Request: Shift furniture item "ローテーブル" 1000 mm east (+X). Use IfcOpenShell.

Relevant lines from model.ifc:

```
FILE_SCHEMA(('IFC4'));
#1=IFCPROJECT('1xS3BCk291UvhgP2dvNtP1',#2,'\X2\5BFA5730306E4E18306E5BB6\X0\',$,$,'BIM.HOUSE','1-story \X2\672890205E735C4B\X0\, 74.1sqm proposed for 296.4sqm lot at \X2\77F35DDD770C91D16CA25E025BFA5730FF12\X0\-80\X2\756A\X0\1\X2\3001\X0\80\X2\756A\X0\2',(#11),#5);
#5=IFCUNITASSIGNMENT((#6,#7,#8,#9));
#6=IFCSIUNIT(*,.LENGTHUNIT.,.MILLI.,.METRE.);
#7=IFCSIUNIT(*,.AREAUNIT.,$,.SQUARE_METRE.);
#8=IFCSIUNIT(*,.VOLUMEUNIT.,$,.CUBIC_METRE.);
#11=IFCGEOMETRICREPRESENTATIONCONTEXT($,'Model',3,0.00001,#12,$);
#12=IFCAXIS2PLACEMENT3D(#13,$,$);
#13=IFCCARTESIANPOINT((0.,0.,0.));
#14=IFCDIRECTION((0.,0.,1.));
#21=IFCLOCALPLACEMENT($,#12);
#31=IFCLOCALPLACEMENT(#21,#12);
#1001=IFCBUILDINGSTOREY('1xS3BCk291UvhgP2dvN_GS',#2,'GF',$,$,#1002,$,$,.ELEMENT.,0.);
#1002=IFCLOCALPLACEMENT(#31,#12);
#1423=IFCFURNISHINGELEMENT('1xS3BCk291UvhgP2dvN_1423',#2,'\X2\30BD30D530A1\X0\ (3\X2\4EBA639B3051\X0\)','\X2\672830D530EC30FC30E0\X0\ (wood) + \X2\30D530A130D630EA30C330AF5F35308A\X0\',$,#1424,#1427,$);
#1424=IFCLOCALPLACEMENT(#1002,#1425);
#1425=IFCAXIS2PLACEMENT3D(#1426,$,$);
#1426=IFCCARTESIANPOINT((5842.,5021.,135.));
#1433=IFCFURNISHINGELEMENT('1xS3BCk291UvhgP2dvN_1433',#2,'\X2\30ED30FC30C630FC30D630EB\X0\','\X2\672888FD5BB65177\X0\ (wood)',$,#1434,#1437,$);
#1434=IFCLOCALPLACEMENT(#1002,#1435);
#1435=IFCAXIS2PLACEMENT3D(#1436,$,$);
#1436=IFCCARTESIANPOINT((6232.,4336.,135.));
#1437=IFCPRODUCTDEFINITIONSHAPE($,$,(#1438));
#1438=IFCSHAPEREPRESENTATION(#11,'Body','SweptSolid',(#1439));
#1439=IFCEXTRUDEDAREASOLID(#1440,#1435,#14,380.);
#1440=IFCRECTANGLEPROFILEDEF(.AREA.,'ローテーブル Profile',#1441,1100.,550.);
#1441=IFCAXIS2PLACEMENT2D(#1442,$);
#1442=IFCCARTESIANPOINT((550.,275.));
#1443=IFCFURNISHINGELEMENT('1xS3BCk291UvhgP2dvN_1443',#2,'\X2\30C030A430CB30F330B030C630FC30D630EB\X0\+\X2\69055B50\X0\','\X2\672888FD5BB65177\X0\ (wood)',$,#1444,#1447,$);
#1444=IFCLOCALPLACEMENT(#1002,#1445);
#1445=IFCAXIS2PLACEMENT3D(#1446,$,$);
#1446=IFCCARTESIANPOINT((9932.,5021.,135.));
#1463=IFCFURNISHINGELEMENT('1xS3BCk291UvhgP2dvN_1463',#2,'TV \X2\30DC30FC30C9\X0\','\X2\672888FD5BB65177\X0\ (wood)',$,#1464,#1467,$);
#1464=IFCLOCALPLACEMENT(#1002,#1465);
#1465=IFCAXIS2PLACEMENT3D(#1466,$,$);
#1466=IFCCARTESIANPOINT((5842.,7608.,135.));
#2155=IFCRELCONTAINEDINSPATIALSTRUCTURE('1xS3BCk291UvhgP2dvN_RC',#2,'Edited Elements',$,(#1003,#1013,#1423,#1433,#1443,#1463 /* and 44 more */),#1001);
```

```python
import ifcopenshell
import ifcopenshell.api.geometry
import ifcopenshell.util.placement

model = ifcopenshell.open("model.ifc")

item = model.by_guid("1xS3BCk291UvhgP2dvN_1433")
matrix = ifcopenshell.util.placement.get_local_placement(item.ObjectPlacement)
matrix[0, 3] += 1000.0
ifcopenshell.api.geometry.edit_object_placement(model, product=item, matrix=matrix, is_si=False)

print(ifcopenshell.util.placement.get_local_placement(item.ObjectPlacement).round(3) + 0.0)

model.write("model_updated.ifc")
```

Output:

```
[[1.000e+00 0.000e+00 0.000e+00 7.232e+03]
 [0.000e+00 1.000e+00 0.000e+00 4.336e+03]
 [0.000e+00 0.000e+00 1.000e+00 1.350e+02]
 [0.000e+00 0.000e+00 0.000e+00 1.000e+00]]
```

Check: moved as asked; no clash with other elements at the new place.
